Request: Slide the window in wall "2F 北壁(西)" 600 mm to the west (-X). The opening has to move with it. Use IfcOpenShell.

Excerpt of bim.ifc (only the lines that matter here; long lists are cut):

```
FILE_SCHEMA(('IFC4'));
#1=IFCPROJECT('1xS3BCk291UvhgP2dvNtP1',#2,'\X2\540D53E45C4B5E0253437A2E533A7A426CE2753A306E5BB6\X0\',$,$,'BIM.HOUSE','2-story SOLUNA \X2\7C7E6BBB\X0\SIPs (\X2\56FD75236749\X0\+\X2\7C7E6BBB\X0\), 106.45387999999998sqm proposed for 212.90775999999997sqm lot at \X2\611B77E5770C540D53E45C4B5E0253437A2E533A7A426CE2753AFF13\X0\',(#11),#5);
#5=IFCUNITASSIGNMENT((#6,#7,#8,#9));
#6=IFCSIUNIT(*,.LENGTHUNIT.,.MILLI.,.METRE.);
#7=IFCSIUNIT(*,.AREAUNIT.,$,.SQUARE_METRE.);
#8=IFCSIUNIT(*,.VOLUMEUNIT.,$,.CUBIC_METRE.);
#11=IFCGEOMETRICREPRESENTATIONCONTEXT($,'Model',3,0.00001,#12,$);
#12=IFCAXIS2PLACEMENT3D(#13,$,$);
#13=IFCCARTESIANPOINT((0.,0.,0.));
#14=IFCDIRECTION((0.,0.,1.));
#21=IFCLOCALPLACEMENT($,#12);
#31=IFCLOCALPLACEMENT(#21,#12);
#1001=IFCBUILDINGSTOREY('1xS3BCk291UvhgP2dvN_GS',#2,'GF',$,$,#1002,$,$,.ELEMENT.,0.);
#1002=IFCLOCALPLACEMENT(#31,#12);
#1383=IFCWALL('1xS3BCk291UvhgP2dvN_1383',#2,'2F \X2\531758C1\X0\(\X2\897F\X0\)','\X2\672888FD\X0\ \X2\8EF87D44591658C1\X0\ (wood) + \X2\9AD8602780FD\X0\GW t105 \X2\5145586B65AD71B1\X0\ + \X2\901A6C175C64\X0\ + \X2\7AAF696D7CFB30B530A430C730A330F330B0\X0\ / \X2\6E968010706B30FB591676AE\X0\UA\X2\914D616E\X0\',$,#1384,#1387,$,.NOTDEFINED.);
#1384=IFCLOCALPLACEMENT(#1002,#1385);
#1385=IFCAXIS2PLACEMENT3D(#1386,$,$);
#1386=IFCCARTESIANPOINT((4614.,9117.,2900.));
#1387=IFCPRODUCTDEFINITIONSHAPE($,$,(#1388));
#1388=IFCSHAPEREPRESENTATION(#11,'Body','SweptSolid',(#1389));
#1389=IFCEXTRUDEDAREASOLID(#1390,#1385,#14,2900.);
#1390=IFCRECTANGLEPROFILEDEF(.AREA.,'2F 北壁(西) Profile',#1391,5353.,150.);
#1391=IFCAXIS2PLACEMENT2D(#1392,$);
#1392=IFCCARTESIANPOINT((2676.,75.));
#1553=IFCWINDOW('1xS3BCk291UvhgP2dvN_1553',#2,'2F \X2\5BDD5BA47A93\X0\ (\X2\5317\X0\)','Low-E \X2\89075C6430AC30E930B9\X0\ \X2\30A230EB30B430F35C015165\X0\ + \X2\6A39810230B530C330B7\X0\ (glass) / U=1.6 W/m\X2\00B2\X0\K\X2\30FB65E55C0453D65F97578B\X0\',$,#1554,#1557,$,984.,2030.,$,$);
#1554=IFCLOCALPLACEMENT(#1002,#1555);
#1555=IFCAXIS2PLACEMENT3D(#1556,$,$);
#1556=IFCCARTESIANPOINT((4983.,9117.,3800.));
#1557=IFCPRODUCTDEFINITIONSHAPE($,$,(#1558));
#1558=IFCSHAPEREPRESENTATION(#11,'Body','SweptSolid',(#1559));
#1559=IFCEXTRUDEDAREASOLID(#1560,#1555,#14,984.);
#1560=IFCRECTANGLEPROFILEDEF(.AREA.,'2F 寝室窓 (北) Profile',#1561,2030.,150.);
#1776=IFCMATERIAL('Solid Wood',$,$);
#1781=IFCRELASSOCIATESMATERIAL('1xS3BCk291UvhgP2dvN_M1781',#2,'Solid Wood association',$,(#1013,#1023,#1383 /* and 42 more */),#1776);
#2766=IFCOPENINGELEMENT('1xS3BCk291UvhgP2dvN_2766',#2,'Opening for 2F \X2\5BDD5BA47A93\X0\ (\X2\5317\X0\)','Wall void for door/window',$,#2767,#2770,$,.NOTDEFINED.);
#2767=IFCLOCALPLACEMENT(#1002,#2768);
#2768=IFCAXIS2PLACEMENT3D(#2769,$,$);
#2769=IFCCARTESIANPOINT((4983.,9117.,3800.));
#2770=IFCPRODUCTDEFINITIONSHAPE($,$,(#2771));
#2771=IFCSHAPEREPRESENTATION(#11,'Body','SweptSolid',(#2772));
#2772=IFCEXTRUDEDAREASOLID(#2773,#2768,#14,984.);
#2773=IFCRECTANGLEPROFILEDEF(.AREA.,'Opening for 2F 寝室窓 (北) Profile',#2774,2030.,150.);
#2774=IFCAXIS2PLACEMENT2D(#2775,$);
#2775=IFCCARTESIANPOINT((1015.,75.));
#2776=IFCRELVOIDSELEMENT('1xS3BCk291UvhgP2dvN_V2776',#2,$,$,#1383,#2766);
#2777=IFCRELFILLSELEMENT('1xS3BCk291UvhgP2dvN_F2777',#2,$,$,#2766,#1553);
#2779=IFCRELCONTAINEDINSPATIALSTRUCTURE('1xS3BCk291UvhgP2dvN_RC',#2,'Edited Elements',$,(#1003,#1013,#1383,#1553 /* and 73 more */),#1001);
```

```python
import ifcopenshell
import ifcopenshell.api.geometry
import ifcopenshell.util.placement

model = ifcopenshell.open("bim.ifc")

window = model.by_guid("1xS3BCk291UvhgP2dvN_1553")
opening = window.FillsVoids[0].RelatingOpeningElement
wall = opening.VoidsElements[0].RelatingBuildingElement

wall_matrix = ifcopenshell.util.placement.get_local_placement(wall.ObjectPlacement)
shift = wall_matrix[:3, 0] * -600.0
before = ifcopenshell.util.placement.get_local_placement(window.ObjectPlacement)[:3, 3].copy()

# The window is not placed relative to its opening, so move both.
for product in (opening, window):
    matrix = ifcopenshell.util.placement.get_local_placement(product.ObjectPlacement)
    matrix[:3, 3] += shift
    ifcopenshell.api.geometry.edit_object_placement(model, product=product, matrix=matrix, is_si=False)

after = ifcopenshell.util.placement.get_local_placement(window.ObjectPlacement)[:3, 3]
print("window moved by", (after - before).round(3) + 0.0)

model.write("bim-out.ifc")
```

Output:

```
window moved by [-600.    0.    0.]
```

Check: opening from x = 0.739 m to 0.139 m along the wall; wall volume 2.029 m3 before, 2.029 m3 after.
